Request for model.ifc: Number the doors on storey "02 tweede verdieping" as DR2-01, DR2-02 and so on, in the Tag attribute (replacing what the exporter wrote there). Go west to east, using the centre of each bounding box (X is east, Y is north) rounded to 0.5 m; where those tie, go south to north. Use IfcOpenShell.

First a look at what the model holds.

```python
import ifcopenshell
import ifcopenshell.util.element
import ifcopenshell.util.placement

model = ifcopenshell.open("model.ifc")
print(model.schema)
storey = next(s for s in model.by_type("IfcBuildingStorey") if s.Name == "02 tweede verdieping")
doors = [e for e in ifcopenshell.util.element.get_decomposition(storey) if e.is_a("IfcDoor")]
for e in sorted(doors, key=lambda e: e.id()):
    origin = ifcopenshell.util.placement.get_local_placement(e.ObjectPlacement)[:3, 3]
    print(e.id(), e.Tag, e.Name, origin.round(2) + 0.0, sep=" | ")
```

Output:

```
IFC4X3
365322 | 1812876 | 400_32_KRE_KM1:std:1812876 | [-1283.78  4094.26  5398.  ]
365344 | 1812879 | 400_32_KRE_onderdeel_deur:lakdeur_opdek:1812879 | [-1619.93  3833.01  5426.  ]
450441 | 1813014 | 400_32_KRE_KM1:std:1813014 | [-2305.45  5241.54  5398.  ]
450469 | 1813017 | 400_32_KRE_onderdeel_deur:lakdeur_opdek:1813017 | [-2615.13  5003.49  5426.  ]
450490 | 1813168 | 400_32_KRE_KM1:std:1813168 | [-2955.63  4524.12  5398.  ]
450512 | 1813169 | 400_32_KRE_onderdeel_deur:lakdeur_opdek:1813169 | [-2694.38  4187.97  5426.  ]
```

```python
import ifcopenshell
import ifcopenshell.geom
import ifcopenshell.util.element
import ifcopenshell.util.shape

model = ifcopenshell.open("model.ifc")
settings = ifcopenshell.geom.settings()
settings.set("use-world-coords", True)


def centre(element):
    shape = ifcopenshell.geom.create_shape(settings, element)
    return ifcopenshell.util.shape.get_bbox_centroid(shape.geometry)


storey = next(s for s in model.by_type("IfcBuildingStorey") if s.Name == "02 tweede verdieping")
doors = [e for e in ifcopenshell.util.element.get_decomposition(storey) if e.is_a("IfcDoor")]

# Insertion points can sit at a corner or the storey origin, so sort by the geometry (in metres).
centres = {e: centre(e) for e in doors}
doors.sort(key=lambda e: (round(centres[e][0] / 0.5), centres[e][1]))

for i, e in enumerate(doors, start=1):
    number = f"DR2-{i:02d}"
    e.Tag = number
    print(e.id(), number)

model.write("model_edited.ifc")
```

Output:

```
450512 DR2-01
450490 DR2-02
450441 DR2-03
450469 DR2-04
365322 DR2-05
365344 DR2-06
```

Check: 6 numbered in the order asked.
